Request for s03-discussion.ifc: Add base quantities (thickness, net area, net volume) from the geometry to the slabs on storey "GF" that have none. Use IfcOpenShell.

First a look at what the model holds.

```python
import ifcopenshell
import ifcopenshell.util.element
import ifcopenshell.util.unit

model = ifcopenshell.open("s03-discussion.ifc")
print(model.schema)
for unit_type in ("LENGTHUNIT", "AREAUNIT", "VOLUMEUNIT"):
    print(unit_type, ifcopenshell.util.unit.calculate_unit_scale(model, unit_type))
storey = next(s for s in model.by_type("IfcBuildingStorey") if s.Name == "GF")
slabs = [e for e in ifcopenshell.util.element.get_decomposition(storey) if e.is_a("IfcSlab")]
for e in sorted(slabs, key=lambda e: e.id()):
    print(e.id(), e.is_a(), e.Name, list(ifcopenshell.util.element.get_psets(e, qtos_only=True)), sep=" | ")
```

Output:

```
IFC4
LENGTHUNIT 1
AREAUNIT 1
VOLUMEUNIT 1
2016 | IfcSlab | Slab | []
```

```python
import ifcopenshell
import ifcopenshell.api.pset
import ifcopenshell.geom
import ifcopenshell.util.element
import ifcopenshell.util.shape
import ifcopenshell.util.unit

model = ifcopenshell.open("s03-discussion.ifc")
unit_scale = ifcopenshell.util.unit.calculate_unit_scale(model)
area_scale = ifcopenshell.util.unit.calculate_unit_scale(model, "AREAUNIT")
volume_scale = ifcopenshell.util.unit.calculate_unit_scale(model, "VOLUMEUNIT")
settings = ifcopenshell.geom.settings()

storey = next(s for s in model.by_type("IfcBuildingStorey") if s.Name == "GF")
slabs = [e for e in ifcopenshell.util.element.get_decomposition(storey) if e.is_a("IfcSlab")]

for e in sorted(slabs, key=lambda e: e.id()):
    if ifcopenshell.util.element.get_psets(e, qtos_only=True, should_inherit=False):
        continue
    # Geometry comes back in metres, in the element's own axes.
    shape = ifcopenshell.geom.create_shape(settings, e)
    values = {
        "Width": ifcopenshell.util.shape.get_z(shape.geometry) / unit_scale,
        "NetArea": ifcopenshell.util.shape.get_footprint_area(shape.geometry) / area_scale,
        "NetVolume": ifcopenshell.util.shape.get_volume(shape.geometry) / volume_scale,
    }
    qto = ifcopenshell.api.pset.add_qto(model, product=e, name="Qto_SlabBaseQuantities")
    ifcopenshell.api.pset.edit_qto(model, qto=qto, properties=values)
    print(e.id(), {k: round(v, 3) for k, v in values.items()})

model.write("s03-discussion_updated.ifc")
```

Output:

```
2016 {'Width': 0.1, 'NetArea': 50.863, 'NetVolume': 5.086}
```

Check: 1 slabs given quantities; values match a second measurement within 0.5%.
